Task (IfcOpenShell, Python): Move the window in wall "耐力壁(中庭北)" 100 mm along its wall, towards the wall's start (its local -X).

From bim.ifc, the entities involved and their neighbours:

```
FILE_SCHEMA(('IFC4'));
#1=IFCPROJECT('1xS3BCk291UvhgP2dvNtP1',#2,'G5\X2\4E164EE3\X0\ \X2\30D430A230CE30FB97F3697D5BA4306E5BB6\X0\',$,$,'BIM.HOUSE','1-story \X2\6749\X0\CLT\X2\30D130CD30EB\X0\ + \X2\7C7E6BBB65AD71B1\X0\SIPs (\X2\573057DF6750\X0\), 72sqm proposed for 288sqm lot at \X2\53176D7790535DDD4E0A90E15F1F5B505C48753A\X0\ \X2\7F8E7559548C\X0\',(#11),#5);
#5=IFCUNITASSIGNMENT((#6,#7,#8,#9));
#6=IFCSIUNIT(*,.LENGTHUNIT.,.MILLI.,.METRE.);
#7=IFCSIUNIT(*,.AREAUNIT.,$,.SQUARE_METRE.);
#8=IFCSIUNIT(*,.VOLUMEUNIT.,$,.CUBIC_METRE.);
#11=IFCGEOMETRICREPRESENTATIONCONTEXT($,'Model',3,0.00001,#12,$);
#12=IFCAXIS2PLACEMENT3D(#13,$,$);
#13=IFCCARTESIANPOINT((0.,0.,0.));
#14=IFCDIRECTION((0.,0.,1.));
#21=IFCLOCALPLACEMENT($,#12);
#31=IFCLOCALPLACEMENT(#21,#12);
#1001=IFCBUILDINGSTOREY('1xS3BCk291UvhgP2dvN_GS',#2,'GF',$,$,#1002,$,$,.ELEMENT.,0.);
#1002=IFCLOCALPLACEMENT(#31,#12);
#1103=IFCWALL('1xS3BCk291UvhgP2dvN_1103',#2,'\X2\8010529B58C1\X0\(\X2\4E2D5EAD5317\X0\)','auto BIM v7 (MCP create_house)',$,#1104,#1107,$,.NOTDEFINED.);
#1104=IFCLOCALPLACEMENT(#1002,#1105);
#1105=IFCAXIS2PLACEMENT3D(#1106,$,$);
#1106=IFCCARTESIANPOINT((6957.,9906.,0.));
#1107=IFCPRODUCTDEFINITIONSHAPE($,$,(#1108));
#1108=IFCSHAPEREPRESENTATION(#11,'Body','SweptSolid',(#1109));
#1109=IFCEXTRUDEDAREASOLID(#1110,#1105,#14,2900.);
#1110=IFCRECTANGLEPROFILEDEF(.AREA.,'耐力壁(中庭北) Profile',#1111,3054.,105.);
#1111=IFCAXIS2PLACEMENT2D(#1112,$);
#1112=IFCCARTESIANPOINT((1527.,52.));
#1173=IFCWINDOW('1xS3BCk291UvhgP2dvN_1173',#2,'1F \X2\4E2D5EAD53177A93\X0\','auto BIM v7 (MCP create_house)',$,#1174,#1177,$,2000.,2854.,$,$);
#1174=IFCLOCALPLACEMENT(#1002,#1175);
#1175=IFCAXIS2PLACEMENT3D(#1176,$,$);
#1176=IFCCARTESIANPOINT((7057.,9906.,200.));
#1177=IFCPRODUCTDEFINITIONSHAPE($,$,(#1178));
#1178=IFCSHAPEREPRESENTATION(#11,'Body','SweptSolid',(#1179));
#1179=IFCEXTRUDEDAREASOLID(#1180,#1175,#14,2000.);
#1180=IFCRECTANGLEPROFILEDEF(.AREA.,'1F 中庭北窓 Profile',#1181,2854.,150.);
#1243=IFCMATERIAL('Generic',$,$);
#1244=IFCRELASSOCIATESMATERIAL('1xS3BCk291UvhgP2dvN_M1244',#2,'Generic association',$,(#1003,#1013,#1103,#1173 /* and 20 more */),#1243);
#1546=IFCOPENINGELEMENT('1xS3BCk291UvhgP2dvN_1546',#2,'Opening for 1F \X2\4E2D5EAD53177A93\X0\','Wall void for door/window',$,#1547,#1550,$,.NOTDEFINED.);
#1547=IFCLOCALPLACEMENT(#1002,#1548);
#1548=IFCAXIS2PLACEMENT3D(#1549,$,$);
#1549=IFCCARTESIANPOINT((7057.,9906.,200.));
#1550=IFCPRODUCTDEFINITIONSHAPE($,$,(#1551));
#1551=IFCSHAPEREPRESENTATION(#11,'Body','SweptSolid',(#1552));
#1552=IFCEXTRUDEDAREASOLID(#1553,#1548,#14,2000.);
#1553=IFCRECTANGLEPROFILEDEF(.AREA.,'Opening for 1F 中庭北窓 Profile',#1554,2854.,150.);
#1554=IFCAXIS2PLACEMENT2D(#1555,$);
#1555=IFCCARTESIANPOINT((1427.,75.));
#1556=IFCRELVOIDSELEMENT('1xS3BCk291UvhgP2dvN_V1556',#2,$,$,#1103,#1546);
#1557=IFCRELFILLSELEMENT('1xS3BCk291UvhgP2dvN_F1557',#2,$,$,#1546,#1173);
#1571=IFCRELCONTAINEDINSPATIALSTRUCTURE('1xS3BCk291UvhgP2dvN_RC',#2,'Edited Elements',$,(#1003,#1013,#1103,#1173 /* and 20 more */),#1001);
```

```python
import ifcopenshell
import ifcopenshell.api.geometry
import ifcopenshell.util.placement

model = ifcopenshell.open("bim.ifc")

window = model.by_guid("1xS3BCk291UvhgP2dvN_1173")
opening = window.FillsVoids[0].RelatingOpeningElement
wall = opening.VoidsElements[0].RelatingBuildingElement

wall_matrix = ifcopenshell.util.placement.get_local_placement(wall.ObjectPlacement)
shift = wall_matrix[:3, 0] * -100.0
before = ifcopenshell.util.placement.get_local_placement(window.ObjectPlacement)[:3, 3].copy()

# The window is not placed relative to its opening, so move both.
for product in (opening, window):
    matrix = ifcopenshell.util.placement.get_local_placement(product.ObjectPlacement)
    matrix[:3, 3] += shift
    ifcopenshell.api.geometry.edit_object_placement(model, product=product, matrix=matrix, is_si=False)

after = ifcopenshell.util.placement.get_local_placement(window.ObjectPlacement)[:3, 3]
print("window moved by", (after - before).round(3) + 0.0)

model.write("bim_updated.ifc")
```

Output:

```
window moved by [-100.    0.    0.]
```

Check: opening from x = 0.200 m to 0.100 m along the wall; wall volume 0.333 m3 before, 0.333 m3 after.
